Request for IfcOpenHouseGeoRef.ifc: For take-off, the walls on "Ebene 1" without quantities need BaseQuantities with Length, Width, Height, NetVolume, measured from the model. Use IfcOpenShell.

First a look at what the model holds.

```python
import ifcopenshell
import ifcopenshell.util.element
import ifcopenshell.util.unit

model = ifcopenshell.open("IfcOpenHouseGeoRef.ifc")
print(model.schema)
for unit_type in ("LENGTHUNIT", "AREAUNIT", "VOLUMEUNIT"):
    print(unit_type, ifcopenshell.util.unit.calculate_unit_scale(model, unit_type))
storey = next(s for s in model.by_type("IfcBuildingStorey") if s.Name == "Ebene 1")
walls = [e for e in ifcopenshell.util.element.get_decomposition(storey) if e.is_a("IfcWall")]
for e in sorted(walls, key=lambda e: e.id()):
    print(e.id(), e.is_a(), e.Name, list(ifcopenshell.util.element.get_psets(e, qtos_only=True)), sep=" | ")
```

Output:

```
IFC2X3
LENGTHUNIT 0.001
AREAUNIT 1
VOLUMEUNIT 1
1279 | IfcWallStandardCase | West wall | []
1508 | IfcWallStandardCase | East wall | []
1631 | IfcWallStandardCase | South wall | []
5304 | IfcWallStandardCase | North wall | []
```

```python
import ifcopenshell
import ifcopenshell.api.pset
import ifcopenshell.geom
import ifcopenshell.util.element
import ifcopenshell.util.shape
import ifcopenshell.util.unit

model = ifcopenshell.open("IfcOpenHouseGeoRef.ifc")
unit_scale = ifcopenshell.util.unit.calculate_unit_scale(model)
volume_scale = ifcopenshell.util.unit.calculate_unit_scale(model, "VOLUMEUNIT")
settings = ifcopenshell.geom.settings()

storey = next(s for s in model.by_type("IfcBuildingStorey") if s.Name == "Ebene 1")
walls = [e for e in ifcopenshell.util.element.get_decomposition(storey) if e.is_a("IfcWall")]

for e in sorted(walls, key=lambda e: e.id()):
    if ifcopenshell.util.element.get_psets(e, qtos_only=True, should_inherit=False):
        continue
    # Geometry comes back in metres, in the element's own axes.
    shape = ifcopenshell.geom.create_shape(settings, e)
    values = {
        "Length": ifcopenshell.util.shape.get_x(shape.geometry) / unit_scale,
        "Width": ifcopenshell.util.shape.get_y(shape.geometry) / unit_scale,
        "Height": ifcopenshell.util.shape.get_z(shape.geometry) / unit_scale,
        "NetVolume": ifcopenshell.util.shape.get_volume(shape.geometry) / volume_scale,
    }
    qto = ifcopenshell.api.pset.add_qto(model, product=e, name="BaseQuantities")
    ifcopenshell.api.pset.edit_qto(model, qto=qto, properties=values)
    print(e.id(), {k: round(v, 3) for k, v in values.items()})

model.write("IfcOpenHouseGeoRef_rev.ifc")
```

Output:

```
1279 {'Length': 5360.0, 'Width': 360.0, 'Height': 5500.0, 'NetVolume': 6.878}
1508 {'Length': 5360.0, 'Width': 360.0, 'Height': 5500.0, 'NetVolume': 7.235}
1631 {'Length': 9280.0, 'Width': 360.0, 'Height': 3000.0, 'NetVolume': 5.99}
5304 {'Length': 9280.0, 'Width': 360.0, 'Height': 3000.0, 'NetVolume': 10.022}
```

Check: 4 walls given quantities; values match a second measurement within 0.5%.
